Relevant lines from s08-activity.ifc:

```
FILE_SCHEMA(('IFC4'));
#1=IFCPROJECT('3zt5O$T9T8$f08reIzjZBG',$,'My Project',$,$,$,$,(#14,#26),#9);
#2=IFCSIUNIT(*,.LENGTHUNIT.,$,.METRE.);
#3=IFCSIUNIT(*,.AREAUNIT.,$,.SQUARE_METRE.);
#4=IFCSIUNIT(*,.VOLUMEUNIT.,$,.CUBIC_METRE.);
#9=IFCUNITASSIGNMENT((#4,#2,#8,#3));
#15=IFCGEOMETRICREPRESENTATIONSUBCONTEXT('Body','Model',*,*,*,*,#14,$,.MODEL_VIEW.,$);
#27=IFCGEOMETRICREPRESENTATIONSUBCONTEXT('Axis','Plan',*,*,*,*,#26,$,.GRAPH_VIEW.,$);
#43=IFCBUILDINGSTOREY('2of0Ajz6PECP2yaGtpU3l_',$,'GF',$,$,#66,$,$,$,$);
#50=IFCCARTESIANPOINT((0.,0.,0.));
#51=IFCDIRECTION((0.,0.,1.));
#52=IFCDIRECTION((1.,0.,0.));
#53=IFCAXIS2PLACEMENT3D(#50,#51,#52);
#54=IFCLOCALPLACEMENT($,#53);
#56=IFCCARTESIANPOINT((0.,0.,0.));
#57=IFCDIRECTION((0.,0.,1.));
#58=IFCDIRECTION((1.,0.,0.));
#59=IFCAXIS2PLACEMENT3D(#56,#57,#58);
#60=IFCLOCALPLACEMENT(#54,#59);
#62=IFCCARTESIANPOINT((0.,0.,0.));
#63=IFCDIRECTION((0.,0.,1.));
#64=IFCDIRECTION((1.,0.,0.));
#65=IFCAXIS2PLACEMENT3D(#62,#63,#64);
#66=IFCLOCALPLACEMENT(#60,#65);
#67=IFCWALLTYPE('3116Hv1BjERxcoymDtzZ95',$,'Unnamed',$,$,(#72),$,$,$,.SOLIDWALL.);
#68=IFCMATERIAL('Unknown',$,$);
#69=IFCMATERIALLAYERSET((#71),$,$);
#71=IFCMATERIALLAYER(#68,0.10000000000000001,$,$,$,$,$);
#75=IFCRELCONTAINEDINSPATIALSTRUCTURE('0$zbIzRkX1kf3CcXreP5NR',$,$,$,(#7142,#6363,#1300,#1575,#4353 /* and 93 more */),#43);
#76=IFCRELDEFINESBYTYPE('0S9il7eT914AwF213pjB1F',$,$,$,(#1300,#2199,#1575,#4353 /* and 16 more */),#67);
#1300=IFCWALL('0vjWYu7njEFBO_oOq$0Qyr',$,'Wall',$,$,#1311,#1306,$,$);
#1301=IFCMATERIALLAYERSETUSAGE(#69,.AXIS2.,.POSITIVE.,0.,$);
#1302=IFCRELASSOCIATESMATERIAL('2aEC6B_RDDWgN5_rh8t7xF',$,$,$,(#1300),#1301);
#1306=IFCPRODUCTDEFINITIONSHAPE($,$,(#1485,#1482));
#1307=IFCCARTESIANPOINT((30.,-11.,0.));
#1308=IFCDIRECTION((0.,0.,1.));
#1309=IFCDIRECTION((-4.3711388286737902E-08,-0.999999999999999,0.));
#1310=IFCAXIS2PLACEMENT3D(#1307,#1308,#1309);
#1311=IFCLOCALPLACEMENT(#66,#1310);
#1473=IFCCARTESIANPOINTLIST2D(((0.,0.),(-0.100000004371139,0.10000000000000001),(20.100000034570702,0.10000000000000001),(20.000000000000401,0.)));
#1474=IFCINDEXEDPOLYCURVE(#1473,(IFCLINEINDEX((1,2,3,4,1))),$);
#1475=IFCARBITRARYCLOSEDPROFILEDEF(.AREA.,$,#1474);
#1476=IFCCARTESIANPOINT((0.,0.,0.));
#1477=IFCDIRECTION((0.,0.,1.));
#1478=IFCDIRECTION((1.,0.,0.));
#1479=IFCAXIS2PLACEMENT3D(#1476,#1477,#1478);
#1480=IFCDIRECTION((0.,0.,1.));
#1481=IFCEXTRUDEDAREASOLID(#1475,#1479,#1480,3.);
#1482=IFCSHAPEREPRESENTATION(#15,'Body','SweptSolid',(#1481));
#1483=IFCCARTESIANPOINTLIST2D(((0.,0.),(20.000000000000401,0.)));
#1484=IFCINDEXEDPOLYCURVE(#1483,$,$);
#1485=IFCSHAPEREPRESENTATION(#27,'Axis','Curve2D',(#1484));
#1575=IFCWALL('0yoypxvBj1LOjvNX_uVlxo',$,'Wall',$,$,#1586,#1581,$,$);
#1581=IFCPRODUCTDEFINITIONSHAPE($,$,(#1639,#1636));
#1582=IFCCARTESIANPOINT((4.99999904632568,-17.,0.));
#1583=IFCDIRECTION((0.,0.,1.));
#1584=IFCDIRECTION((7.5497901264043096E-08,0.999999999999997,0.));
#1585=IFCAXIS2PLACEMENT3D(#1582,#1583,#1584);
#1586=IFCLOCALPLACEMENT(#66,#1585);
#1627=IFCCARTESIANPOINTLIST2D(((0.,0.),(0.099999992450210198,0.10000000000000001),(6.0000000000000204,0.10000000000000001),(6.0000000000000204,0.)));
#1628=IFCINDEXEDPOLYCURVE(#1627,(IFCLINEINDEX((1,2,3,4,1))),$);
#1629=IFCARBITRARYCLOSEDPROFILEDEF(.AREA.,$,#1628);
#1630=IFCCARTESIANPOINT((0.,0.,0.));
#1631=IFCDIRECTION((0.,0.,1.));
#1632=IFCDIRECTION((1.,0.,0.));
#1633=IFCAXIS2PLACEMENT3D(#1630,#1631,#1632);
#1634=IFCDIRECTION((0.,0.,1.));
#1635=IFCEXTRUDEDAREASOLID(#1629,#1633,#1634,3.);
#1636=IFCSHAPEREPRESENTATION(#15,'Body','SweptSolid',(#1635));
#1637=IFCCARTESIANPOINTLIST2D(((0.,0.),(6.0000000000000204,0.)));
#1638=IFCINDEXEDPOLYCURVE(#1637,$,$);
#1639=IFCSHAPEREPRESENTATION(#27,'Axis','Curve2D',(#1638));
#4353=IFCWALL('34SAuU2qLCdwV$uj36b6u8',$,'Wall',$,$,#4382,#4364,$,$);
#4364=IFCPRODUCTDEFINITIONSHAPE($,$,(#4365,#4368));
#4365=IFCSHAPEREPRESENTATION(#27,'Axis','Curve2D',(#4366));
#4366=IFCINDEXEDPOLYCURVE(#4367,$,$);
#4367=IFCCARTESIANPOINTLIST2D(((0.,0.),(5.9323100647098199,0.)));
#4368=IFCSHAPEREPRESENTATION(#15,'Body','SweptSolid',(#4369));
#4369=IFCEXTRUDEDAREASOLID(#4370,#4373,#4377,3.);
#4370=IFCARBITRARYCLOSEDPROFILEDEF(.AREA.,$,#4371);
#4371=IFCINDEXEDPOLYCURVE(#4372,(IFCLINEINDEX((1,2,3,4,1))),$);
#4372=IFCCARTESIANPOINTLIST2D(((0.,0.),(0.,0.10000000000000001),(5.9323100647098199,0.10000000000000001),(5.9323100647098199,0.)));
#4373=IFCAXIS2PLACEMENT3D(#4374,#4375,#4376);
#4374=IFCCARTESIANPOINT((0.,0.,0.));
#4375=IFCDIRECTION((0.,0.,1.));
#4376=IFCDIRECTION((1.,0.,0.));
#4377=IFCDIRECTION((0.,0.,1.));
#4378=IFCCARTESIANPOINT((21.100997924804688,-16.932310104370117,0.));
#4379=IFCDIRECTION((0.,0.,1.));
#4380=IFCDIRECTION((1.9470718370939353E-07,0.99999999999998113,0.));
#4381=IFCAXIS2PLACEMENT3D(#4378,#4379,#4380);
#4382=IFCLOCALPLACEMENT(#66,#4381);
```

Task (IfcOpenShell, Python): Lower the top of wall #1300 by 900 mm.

```python
import ifcopenshell
import ifcopenshell.geom
import ifcopenshell.util.representation
import ifcopenshell.util.shape
import ifcopenshell.util.unit

model = ifcopenshell.open("s08-activity.ifc")
unit_scale = ifcopenshell.util.unit.calculate_unit_scale(model)
settings = ifcopenshell.geom.settings()


def volume(element):
    """Net volume in cubic metres, openings subtracted."""
    shape = ifcopenshell.geom.create_shape(settings, element)
    return ifcopenshell.util.shape.get_volume(shape.geometry)


wall = model.by_id(1300)
before = volume(wall)

body = ifcopenshell.util.representation.get_representation(wall, "Model", "Body")
solid = body.Items[0]
old_height = solid.Depth
solid.Depth -= 0.9 / unit_scale
after = volume(wall)

print(f"height {old_height:g} -> {solid.Depth:g}, volume {before:.3f} -> {after:.3f} m3")

model.write("s08-activity_edited.ifc")
```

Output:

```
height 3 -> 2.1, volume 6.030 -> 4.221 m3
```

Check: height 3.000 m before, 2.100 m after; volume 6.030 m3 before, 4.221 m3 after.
